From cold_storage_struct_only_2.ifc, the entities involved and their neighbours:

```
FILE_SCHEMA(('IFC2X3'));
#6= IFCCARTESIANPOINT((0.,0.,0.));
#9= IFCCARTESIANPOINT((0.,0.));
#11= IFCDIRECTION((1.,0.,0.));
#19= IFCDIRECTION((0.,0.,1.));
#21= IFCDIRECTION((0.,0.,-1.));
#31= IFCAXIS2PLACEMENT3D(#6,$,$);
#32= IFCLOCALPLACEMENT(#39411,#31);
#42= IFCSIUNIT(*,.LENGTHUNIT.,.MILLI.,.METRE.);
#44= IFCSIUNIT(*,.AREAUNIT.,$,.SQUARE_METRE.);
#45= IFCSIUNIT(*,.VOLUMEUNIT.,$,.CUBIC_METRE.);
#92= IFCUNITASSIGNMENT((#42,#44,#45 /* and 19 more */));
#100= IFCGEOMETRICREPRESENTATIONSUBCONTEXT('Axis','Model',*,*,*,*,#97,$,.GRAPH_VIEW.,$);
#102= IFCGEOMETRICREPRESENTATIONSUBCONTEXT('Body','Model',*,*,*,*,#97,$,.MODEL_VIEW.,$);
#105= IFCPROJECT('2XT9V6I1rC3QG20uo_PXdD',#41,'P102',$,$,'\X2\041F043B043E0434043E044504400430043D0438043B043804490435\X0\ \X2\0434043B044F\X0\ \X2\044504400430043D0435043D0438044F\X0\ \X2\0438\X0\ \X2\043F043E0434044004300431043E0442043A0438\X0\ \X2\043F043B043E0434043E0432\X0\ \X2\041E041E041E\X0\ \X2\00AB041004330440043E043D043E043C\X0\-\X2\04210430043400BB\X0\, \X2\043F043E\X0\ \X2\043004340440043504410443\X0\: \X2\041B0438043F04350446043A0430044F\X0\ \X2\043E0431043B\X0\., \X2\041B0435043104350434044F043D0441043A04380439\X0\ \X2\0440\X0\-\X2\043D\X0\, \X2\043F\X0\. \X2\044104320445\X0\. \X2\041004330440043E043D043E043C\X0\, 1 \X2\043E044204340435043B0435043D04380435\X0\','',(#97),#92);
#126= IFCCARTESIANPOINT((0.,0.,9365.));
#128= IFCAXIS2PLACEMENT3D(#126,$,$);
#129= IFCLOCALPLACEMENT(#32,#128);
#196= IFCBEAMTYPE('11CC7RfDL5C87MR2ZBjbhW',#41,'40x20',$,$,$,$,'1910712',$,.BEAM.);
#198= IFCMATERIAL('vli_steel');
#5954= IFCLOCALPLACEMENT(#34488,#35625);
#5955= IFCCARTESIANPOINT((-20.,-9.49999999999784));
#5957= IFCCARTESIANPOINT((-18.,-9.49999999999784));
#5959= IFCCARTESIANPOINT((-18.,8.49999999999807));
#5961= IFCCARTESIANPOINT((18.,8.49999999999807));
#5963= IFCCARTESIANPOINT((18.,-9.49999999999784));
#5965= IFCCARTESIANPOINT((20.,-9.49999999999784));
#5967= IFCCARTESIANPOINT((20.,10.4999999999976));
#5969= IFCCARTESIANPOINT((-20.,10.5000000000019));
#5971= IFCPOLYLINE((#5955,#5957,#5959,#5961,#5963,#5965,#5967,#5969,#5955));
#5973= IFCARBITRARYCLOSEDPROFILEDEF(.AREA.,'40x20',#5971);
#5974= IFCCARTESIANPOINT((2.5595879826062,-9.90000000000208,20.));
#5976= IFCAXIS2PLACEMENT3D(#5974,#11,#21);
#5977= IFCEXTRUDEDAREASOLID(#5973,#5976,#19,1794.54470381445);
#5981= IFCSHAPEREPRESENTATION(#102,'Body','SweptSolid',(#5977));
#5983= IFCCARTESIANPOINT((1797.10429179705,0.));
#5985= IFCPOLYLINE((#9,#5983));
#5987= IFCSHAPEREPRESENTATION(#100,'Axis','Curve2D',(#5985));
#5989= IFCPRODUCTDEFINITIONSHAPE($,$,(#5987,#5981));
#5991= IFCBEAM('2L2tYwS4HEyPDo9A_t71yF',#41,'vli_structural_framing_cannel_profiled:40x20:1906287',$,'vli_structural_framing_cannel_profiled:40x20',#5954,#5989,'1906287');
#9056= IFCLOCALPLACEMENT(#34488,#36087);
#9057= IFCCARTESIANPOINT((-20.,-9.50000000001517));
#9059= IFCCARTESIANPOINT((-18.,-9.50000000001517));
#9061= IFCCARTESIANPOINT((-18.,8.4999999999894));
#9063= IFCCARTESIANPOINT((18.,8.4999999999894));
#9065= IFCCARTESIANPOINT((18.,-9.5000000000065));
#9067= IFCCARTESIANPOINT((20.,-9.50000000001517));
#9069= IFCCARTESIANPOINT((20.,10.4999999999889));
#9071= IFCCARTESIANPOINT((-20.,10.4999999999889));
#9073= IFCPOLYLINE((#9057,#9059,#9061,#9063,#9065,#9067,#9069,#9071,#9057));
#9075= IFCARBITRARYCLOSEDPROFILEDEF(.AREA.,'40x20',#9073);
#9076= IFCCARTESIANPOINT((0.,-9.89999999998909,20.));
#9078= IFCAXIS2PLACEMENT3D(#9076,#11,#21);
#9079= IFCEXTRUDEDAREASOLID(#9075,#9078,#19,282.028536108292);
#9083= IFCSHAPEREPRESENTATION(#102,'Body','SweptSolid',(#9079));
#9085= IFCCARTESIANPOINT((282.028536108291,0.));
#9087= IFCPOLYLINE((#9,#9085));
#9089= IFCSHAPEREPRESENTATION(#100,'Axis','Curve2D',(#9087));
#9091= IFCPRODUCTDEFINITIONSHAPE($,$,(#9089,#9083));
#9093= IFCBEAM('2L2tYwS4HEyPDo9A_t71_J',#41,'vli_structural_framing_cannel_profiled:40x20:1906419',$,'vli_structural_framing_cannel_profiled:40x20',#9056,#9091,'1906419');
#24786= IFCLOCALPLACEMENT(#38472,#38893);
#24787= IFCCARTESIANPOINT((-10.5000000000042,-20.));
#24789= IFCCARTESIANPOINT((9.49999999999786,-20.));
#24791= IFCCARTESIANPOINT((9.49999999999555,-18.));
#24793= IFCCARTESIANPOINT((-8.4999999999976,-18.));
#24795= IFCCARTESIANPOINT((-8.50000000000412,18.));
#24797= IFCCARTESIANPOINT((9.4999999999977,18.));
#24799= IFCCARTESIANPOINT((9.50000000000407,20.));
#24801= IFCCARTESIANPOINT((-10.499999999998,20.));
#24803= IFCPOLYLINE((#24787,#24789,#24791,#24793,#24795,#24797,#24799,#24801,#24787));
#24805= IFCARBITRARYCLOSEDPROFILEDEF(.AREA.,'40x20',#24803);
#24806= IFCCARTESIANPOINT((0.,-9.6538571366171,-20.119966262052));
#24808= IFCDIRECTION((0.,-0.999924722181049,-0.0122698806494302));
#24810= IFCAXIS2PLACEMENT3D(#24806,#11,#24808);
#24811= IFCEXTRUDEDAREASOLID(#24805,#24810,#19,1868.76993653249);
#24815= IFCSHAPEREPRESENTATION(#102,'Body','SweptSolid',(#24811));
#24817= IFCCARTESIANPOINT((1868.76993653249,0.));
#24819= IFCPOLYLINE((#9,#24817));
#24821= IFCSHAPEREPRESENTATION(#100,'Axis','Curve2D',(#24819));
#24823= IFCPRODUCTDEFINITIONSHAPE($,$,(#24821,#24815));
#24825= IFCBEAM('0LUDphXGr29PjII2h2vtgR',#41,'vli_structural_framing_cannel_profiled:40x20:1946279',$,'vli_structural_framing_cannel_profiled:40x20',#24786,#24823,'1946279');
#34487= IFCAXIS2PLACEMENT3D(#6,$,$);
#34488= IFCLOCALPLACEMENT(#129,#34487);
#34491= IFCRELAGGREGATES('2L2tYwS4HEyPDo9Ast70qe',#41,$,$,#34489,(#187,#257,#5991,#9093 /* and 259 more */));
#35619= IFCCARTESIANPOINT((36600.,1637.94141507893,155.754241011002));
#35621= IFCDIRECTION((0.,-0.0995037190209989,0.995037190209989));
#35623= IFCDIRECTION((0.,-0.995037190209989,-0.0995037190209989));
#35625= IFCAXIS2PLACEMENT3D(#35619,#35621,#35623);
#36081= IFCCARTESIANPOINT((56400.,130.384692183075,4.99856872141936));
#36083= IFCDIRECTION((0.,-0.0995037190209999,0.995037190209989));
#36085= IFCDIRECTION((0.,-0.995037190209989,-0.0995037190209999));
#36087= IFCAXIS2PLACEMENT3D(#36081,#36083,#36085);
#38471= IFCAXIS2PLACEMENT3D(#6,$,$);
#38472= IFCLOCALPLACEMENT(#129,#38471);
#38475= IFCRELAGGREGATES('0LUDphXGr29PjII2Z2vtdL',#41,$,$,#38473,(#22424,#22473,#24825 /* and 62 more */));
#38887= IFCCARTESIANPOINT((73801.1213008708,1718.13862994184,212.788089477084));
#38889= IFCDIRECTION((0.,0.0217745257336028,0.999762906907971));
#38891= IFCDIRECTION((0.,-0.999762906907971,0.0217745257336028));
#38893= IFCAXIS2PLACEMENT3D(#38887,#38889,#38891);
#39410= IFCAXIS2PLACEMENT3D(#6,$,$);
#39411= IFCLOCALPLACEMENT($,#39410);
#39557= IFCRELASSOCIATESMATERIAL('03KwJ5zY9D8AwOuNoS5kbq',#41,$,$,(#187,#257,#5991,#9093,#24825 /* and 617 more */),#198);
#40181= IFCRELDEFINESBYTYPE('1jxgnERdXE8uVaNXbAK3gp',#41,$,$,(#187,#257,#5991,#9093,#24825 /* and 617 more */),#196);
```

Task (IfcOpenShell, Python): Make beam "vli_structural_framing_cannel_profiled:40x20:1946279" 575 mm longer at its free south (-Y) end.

```python
import numpy as np
import ifcopenshell
import ifcopenshell.util.representation

model = ifcopenshell.open("cold_storage_struct_only_2.ifc")

member = model.by_guid("0LUDphXGr29PjII2h2vtgR")
change = 575.0

# The extrusion runs towards the end named, so only its depth changes.
body = ifcopenshell.util.representation.get_representation(member, "Model", "Body")
solid = body.Items[0]
old_length = solid.Depth
solid.Depth += change

# Move the axis end point with it.
axis = next(r for r in member.Representation.Representations if r.RepresentationIdentifier == "Axis").Items[0]
start, end = (np.array(p.Coordinates) for p in axis.Points)
end = end + (end - start) / np.linalg.norm(end - start) * change
point = model.createIfcCartesianPoint(end.tolist())
axis.Points = [axis.Points[0], point]

print(f"length {old_length:g} -> {solid.Depth:g}")

model.write("cold_storage_struct_only_2_updated.ifc")
```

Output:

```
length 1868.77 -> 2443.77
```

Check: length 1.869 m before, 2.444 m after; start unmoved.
